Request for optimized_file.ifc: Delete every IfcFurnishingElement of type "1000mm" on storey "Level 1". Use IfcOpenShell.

First a look at what the model holds.

```python
import ifcopenshell
import ifcopenshell.util.element

model = ifcopenshell.open("optimized_file.ifc")
print(model.schema)
storey = next(s for s in model.by_type("IfcBuildingStorey") if s.Name == "Level 1")
furniture = [e for e in ifcopenshell.util.element.get_decomposition(storey) if e.is_a("IfcFurnishingElement")]
seen = {}
for e in furniture:
    element_type = ifcopenshell.util.element.get_type(e)
    name = element_type.Name if element_type not in (None, e) else None
    seen[name] = seen.get(name, 0) + 1
for name, count in sorted(seen.items(), key=str):
    print(count, "x", name)
```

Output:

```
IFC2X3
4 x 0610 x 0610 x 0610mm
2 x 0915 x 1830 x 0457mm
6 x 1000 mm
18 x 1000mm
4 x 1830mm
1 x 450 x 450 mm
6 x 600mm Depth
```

```python
import ifcopenshell
import ifcopenshell.api.root
import ifcopenshell.util.element

model = ifcopenshell.open("optimized_file.ifc")

storey = next(s for s in model.by_type("IfcBuildingStorey") if s.Name == "Level 1")
furniture = [e for e in ifcopenshell.util.element.get_decomposition(storey) if e.is_a("IfcFurnishingElement")]
targets = [e for e in furniture if (t := ifcopenshell.util.element.get_type(e)) not in (None, e) and t.Name == "1000mm"]

for e in targets:
    ifcopenshell.api.root.remove_product(model, product=e)
print(len(targets), "removed")

model.write("optimized_file_v2.ifc")
```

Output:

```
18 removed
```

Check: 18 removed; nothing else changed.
